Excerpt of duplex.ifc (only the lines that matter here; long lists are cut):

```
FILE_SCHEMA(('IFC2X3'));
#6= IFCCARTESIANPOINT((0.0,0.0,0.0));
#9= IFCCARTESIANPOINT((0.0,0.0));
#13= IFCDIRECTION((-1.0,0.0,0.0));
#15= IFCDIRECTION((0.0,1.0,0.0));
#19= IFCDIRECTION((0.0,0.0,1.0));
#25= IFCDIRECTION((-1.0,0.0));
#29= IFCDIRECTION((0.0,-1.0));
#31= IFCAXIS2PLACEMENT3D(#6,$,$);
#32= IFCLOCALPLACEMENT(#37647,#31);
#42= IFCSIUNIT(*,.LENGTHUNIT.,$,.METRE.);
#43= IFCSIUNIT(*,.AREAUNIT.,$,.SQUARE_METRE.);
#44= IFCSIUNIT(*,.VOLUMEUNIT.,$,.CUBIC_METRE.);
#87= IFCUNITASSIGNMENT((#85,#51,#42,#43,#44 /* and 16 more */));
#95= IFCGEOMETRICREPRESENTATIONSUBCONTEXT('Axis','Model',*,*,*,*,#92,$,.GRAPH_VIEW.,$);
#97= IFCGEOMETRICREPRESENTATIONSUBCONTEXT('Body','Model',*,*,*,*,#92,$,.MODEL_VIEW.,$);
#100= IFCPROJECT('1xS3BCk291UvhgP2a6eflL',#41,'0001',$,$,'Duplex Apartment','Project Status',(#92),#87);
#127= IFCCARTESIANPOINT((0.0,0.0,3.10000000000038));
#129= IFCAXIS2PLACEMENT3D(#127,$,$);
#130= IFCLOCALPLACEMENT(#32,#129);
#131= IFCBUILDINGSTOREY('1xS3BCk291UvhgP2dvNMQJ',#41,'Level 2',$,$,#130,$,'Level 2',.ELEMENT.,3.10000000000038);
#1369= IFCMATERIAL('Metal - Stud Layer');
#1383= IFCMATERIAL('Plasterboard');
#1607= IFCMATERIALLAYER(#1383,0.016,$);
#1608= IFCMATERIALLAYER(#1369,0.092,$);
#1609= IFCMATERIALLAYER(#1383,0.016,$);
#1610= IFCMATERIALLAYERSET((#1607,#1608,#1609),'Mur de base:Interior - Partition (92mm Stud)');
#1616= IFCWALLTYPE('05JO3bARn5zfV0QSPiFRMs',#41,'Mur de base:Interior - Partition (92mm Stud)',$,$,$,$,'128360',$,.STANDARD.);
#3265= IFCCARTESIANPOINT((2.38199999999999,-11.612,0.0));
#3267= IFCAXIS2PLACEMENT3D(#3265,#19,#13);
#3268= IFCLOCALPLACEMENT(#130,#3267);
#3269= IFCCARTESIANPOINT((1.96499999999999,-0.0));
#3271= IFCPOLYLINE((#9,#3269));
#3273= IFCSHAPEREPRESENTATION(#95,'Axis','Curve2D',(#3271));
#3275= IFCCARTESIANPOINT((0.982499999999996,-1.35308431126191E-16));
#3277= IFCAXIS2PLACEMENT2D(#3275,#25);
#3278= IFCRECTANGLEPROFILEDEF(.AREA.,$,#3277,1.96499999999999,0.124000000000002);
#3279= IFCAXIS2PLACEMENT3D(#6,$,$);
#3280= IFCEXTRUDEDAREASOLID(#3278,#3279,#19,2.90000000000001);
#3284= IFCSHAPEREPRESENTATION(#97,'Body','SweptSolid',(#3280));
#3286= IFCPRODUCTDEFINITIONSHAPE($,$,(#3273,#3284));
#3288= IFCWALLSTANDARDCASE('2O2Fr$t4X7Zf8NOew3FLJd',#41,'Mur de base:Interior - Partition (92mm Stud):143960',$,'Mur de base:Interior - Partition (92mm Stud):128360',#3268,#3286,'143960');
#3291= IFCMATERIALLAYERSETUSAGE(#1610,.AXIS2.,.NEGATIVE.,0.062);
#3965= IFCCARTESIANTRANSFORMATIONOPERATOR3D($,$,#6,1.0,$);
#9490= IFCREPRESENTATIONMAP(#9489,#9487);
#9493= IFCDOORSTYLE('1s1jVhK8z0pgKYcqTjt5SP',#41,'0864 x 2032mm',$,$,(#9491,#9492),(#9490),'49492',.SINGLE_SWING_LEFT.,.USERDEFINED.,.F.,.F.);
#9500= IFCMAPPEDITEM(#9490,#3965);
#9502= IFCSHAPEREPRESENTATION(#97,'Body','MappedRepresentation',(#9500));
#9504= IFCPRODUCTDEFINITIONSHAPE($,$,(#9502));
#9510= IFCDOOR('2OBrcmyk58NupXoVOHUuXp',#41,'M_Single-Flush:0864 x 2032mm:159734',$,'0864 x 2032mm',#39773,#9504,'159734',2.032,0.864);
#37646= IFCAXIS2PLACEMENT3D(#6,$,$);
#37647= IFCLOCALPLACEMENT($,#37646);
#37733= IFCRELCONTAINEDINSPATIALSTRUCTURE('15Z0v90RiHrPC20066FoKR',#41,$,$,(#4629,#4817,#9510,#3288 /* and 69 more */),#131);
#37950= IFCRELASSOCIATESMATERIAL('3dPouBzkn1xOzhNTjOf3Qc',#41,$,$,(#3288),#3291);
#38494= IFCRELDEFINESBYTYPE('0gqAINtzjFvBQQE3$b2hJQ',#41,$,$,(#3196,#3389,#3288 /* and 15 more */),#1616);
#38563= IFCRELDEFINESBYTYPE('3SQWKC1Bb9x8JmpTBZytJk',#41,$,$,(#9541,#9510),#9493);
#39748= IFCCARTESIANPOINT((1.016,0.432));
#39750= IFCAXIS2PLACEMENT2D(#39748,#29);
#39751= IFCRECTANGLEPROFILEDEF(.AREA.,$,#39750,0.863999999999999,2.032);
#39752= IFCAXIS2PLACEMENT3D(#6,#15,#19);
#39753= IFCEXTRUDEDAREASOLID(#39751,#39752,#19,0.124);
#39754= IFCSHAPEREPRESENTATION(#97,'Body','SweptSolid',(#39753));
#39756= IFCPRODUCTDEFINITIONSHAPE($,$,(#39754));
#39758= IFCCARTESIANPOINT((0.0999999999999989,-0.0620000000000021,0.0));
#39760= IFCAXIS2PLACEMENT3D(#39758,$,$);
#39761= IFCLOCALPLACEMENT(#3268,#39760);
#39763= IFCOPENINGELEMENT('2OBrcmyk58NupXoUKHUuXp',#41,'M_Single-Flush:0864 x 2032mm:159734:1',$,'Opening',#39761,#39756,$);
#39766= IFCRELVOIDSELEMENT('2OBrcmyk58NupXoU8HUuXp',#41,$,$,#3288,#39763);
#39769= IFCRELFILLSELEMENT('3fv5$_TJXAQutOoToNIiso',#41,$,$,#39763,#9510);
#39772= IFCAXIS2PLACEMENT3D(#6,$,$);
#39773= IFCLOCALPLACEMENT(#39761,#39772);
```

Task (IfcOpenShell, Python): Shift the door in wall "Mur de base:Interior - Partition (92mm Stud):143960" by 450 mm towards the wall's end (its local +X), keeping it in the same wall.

```python
import ifcopenshell
import ifcopenshell.api.geometry
import ifcopenshell.util.placement
import ifcopenshell.util.unit

model = ifcopenshell.open("duplex.ifc")
unit_scale = ifcopenshell.util.unit.calculate_unit_scale(model)

door = model.by_guid("2OBrcmyk58NupXoVOHUuXp")
opening = door.FillsVoids[0].RelatingOpeningElement
wall = opening.VoidsElements[0].RelatingBuildingElement

wall_matrix = ifcopenshell.util.placement.get_local_placement(wall.ObjectPlacement)
shift = wall_matrix[:3, 0] * 0.45 / unit_scale
before = ifcopenshell.util.placement.get_local_placement(door.ObjectPlacement)[:3, 3].copy()

# The door is placed relative to its opening, so it follows when the opening moves.
matrix = ifcopenshell.util.placement.get_local_placement(opening.ObjectPlacement)
matrix[:3, 3] += shift
ifcopenshell.api.geometry.edit_object_placement(
    model, product=opening, matrix=matrix, is_si=False, should_transform_children=True
)

after = ifcopenshell.util.placement.get_local_placement(door.ObjectPlacement)[:3, 3]
print("door moved by", (after - before).round(3) + 0.0)

model.write("duplex_updated.ifc")
```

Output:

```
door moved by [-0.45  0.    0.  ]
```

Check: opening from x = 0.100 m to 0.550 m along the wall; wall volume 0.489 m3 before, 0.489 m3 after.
